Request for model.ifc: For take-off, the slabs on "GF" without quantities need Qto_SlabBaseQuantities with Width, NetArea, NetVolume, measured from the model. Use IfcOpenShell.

First a look at what the model holds.

```python
import ifcopenshell
import ifcopenshell.util.element
import ifcopenshell.util.unit

model = ifcopenshell.open("model.ifc")
print(model.schema)
for unit_type in ("LENGTHUNIT", "AREAUNIT", "VOLUMEUNIT"):
    print(unit_type, ifcopenshell.util.unit.calculate_unit_scale(model, unit_type))
storey = next(s for s in model.by_type("IfcBuildingStorey") if s.Name == "GF")
slabs = [e for e in ifcopenshell.util.element.get_decomposition(storey) if e.is_a("IfcSlab")]
for e in sorted(slabs, key=lambda e: e.id()):
    print(e.id(), e.is_a(), e.Name, list(ifcopenshell.util.element.get_psets(e, qtos_only=True)), sep=" | ")
```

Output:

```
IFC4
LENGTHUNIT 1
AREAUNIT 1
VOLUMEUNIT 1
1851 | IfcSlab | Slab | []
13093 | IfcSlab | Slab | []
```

```python
import ifcopenshell
import ifcopenshell.api.pset
import ifcopenshell.geom
import ifcopenshell.util.element
import ifcopenshell.util.shape
import ifcopenshell.util.unit

model = ifcopenshell.open("model.ifc")
unit_scale = ifcopenshell.util.unit.calculate_unit_scale(model)
area_scale = ifcopenshell.util.unit.calculate_unit_scale(model, "AREAUNIT")
volume_scale = ifcopenshell.util.unit.calculate_unit_scale(model, "VOLUMEUNIT")
settings = ifcopenshell.geom.settings()

storey = next(s for s in model.by_type("IfcBuildingStorey") if s.Name == "GF")
slabs = [e for e in ifcopenshell.util.element.get_decomposition(storey) if e.is_a("IfcSlab")]

for e in sorted(slabs, key=lambda e: e.id()):
    if ifcopenshell.util.element.get_psets(e, qtos_only=True, should_inherit=False):
        continue
    # Geometry comes back in metres, in the element's own axes.
    shape = ifcopenshell.geom.create_shape(settings, e)
    values = {
        "Width": ifcopenshell.util.shape.get_z(shape.geometry) / unit_scale,
        "NetArea": ifcopenshell.util.shape.get_footprint_area(shape.geometry) / area_scale,
        "NetVolume": ifcopenshell.util.shape.get_volume(shape.geometry) / volume_scale,
    }
    qto = ifcopenshell.api.pset.add_qto(model, product=e, name="Qto_SlabBaseQuantities")
    ifcopenshell.api.pset.edit_qto(model, qto=qto, properties=values)
    print(e.id(), {k: round(v, 3) for k, v in values.items()})

model.write("model_edited.ifc")
```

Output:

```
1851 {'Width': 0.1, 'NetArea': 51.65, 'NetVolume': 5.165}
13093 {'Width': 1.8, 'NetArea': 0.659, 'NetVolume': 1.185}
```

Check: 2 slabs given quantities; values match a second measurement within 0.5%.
